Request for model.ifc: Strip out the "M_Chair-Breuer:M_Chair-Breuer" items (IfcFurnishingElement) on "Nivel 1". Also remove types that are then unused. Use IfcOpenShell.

First a look at what the model holds.

```python
import ifcopenshell
import ifcopenshell.util.element

model = ifcopenshell.open("model.ifc")
print(model.schema)
storey = next(s for s in model.by_type("IfcBuildingStorey") if s.Name == "Nivel 1")
furniture = [e for e in ifcopenshell.util.element.get_decomposition(storey) if e.is_a("IfcFurnishingElement")]
seen = {}
for e in furniture:
    element_type = ifcopenshell.util.element.get_type(e)
    name = element_type.Name if element_type not in (None, e) else None
    seen[name] = seen.get(name, 0) + 1
for name, count in sorted(seen.items(), key=str):
    print(count, "x", name)
```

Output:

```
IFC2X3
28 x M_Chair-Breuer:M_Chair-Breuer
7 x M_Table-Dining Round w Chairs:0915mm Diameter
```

```python
import ifcopenshell
import ifcopenshell.api.root
import ifcopenshell.util.element

model = ifcopenshell.open("model.ifc")

storey = next(s for s in model.by_type("IfcBuildingStorey") if s.Name == "Nivel 1")
furniture = [e for e in ifcopenshell.util.element.get_decomposition(storey) if e.is_a("IfcFurnishingElement")]
targets = [e for e in furniture if (t := ifcopenshell.util.element.get_type(e)) not in (None, e) and t.Name == "M_Chair-Breuer:M_Chair-Breuer"]
types = {ifcopenshell.util.element.get_type(e) for e in targets} - {None, *targets}

for e in targets:
    ifcopenshell.api.root.remove_product(model, product=e)
print(len(targets), "removed")

unused = [t for t in types if not ifcopenshell.util.element.get_types(t)]
for t in unused:
    ifcopenshell.api.root.remove_product(model, product=t)
print(len(unused), "unused types removed")

model.write("model_v2.ifc")
```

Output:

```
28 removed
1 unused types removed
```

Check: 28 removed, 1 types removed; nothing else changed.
